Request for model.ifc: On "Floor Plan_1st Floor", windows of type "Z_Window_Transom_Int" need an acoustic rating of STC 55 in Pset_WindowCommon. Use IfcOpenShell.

First a look at what the model holds.

```python
import ifcopenshell
import ifcopenshell.util.element

model = ifcopenshell.open("model.ifc")
print(model.schema)
storey = next(s for s in model.by_type("IfcBuildingStorey") if s.Name == "Floor Plan_1st Floor")
windows = [e for e in ifcopenshell.util.element.get_decomposition(storey) if e.is_a("IfcWindow")]
seen = {}
for e in windows:
    element_type = ifcopenshell.util.element.get_type(e)
    key = (element_type.Name if element_type != e and element_type else None, ifcopenshell.util.element.get_pset(e, "Pset_WindowCommon", "AcousticRating"))
    seen[key] = seen.get(key, 0) + 1
for (name, value), count in sorted(seen.items(), key=str):
    print(count, "x", name, "|", value)
```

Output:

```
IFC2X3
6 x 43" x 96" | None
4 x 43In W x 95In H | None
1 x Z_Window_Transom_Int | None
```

```python
import ifcopenshell
import ifcopenshell.api.pset
import ifcopenshell.util.element

model = ifcopenshell.open("model.ifc")

storey = next(s for s in model.by_type("IfcBuildingStorey") if s.Name == "Floor Plan_1st Floor")
windows = [e for e in ifcopenshell.util.element.get_decomposition(storey) if e.is_a("IfcWindow")]

count = 0
for e in windows:
    element_type = ifcopenshell.util.element.get_type(e)
    if element_type in (None, e) or element_type.Name != "Z_Window_Transom_Int":
        continue
    # add_pset returns the element's existing set when there is one.
    pset = ifcopenshell.api.pset.add_pset(model, product=e, name="Pset_WindowCommon")
    ifcopenshell.api.pset.edit_pset(model, pset=pset, properties={"AcousticRating": "STC 55"})
    count += 1

print(count, "windows updated")

model.write("model_edited.ifc")
```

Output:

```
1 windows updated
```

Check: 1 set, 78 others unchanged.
